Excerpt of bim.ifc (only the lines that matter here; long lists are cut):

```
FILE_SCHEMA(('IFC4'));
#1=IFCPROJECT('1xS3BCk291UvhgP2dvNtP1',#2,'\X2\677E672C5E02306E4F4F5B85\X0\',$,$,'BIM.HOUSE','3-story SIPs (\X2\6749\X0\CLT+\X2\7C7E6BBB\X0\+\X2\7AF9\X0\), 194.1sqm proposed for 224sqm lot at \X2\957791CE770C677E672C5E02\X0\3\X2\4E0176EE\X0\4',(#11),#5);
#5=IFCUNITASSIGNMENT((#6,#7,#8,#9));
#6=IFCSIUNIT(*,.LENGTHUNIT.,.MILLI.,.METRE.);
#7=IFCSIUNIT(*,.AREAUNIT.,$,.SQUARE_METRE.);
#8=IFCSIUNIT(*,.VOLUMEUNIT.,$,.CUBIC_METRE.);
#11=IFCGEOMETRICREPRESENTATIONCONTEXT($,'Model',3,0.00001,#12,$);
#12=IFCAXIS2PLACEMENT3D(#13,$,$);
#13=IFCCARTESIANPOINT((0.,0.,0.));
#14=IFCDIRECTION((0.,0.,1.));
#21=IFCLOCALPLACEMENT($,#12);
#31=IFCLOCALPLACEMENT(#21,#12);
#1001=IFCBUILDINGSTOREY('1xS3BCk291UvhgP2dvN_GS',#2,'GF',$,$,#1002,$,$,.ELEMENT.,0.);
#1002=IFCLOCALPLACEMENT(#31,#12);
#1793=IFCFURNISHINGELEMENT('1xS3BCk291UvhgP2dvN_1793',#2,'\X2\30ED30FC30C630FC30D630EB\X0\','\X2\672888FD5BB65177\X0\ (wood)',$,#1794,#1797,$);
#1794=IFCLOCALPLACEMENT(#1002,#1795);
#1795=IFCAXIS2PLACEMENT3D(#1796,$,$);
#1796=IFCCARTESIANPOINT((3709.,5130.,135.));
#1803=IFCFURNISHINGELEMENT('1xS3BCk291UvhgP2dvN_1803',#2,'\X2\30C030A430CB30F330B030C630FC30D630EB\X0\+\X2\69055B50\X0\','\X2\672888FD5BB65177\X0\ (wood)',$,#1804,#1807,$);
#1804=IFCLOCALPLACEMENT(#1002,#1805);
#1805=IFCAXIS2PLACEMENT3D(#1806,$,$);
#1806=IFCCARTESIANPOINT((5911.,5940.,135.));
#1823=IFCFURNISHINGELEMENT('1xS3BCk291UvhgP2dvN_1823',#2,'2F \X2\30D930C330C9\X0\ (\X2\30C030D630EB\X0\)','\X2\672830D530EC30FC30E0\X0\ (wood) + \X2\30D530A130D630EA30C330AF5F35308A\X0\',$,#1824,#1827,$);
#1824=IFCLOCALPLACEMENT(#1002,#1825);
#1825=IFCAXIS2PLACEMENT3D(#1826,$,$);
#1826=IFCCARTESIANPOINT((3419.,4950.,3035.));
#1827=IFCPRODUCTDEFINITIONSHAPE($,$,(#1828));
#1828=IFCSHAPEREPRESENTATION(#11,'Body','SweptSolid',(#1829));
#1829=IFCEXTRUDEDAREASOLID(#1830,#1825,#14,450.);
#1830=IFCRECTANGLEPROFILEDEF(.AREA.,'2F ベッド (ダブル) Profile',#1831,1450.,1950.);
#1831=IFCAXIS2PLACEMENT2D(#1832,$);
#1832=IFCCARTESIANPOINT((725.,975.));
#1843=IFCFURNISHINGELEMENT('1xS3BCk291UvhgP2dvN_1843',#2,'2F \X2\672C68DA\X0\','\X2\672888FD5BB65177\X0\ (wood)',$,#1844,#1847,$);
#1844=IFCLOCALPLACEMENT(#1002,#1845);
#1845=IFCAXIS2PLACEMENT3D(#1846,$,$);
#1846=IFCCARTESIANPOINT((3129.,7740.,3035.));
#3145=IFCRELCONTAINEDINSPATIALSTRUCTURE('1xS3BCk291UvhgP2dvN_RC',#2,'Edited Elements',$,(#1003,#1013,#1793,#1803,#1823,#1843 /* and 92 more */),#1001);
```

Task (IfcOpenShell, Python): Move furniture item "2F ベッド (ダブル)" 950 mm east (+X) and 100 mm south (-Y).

```python
import ifcopenshell
import ifcopenshell.api.geometry
import ifcopenshell.util.placement
import ifcopenshell.util.unit

model = ifcopenshell.open("bim.ifc")
unit_scale = ifcopenshell.util.unit.calculate_unit_scale(model)

item = model.by_guid("1xS3BCk291UvhgP2dvN_1823")
matrix = ifcopenshell.util.placement.get_local_placement(item.ObjectPlacement)
matrix[0, 3] += 0.95 / unit_scale
matrix[1, 3] -= 0.1 / unit_scale
ifcopenshell.api.geometry.edit_object_placement(model, product=item, matrix=matrix, is_si=False)

print(ifcopenshell.util.placement.get_local_placement(item.ObjectPlacement).round(3) + 0.0)

model.write("bim_updated.ifc")
```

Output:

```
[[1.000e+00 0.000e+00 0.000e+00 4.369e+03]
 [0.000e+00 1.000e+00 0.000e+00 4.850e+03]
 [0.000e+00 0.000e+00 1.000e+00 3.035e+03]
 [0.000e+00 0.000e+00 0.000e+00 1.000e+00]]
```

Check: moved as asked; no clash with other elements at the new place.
